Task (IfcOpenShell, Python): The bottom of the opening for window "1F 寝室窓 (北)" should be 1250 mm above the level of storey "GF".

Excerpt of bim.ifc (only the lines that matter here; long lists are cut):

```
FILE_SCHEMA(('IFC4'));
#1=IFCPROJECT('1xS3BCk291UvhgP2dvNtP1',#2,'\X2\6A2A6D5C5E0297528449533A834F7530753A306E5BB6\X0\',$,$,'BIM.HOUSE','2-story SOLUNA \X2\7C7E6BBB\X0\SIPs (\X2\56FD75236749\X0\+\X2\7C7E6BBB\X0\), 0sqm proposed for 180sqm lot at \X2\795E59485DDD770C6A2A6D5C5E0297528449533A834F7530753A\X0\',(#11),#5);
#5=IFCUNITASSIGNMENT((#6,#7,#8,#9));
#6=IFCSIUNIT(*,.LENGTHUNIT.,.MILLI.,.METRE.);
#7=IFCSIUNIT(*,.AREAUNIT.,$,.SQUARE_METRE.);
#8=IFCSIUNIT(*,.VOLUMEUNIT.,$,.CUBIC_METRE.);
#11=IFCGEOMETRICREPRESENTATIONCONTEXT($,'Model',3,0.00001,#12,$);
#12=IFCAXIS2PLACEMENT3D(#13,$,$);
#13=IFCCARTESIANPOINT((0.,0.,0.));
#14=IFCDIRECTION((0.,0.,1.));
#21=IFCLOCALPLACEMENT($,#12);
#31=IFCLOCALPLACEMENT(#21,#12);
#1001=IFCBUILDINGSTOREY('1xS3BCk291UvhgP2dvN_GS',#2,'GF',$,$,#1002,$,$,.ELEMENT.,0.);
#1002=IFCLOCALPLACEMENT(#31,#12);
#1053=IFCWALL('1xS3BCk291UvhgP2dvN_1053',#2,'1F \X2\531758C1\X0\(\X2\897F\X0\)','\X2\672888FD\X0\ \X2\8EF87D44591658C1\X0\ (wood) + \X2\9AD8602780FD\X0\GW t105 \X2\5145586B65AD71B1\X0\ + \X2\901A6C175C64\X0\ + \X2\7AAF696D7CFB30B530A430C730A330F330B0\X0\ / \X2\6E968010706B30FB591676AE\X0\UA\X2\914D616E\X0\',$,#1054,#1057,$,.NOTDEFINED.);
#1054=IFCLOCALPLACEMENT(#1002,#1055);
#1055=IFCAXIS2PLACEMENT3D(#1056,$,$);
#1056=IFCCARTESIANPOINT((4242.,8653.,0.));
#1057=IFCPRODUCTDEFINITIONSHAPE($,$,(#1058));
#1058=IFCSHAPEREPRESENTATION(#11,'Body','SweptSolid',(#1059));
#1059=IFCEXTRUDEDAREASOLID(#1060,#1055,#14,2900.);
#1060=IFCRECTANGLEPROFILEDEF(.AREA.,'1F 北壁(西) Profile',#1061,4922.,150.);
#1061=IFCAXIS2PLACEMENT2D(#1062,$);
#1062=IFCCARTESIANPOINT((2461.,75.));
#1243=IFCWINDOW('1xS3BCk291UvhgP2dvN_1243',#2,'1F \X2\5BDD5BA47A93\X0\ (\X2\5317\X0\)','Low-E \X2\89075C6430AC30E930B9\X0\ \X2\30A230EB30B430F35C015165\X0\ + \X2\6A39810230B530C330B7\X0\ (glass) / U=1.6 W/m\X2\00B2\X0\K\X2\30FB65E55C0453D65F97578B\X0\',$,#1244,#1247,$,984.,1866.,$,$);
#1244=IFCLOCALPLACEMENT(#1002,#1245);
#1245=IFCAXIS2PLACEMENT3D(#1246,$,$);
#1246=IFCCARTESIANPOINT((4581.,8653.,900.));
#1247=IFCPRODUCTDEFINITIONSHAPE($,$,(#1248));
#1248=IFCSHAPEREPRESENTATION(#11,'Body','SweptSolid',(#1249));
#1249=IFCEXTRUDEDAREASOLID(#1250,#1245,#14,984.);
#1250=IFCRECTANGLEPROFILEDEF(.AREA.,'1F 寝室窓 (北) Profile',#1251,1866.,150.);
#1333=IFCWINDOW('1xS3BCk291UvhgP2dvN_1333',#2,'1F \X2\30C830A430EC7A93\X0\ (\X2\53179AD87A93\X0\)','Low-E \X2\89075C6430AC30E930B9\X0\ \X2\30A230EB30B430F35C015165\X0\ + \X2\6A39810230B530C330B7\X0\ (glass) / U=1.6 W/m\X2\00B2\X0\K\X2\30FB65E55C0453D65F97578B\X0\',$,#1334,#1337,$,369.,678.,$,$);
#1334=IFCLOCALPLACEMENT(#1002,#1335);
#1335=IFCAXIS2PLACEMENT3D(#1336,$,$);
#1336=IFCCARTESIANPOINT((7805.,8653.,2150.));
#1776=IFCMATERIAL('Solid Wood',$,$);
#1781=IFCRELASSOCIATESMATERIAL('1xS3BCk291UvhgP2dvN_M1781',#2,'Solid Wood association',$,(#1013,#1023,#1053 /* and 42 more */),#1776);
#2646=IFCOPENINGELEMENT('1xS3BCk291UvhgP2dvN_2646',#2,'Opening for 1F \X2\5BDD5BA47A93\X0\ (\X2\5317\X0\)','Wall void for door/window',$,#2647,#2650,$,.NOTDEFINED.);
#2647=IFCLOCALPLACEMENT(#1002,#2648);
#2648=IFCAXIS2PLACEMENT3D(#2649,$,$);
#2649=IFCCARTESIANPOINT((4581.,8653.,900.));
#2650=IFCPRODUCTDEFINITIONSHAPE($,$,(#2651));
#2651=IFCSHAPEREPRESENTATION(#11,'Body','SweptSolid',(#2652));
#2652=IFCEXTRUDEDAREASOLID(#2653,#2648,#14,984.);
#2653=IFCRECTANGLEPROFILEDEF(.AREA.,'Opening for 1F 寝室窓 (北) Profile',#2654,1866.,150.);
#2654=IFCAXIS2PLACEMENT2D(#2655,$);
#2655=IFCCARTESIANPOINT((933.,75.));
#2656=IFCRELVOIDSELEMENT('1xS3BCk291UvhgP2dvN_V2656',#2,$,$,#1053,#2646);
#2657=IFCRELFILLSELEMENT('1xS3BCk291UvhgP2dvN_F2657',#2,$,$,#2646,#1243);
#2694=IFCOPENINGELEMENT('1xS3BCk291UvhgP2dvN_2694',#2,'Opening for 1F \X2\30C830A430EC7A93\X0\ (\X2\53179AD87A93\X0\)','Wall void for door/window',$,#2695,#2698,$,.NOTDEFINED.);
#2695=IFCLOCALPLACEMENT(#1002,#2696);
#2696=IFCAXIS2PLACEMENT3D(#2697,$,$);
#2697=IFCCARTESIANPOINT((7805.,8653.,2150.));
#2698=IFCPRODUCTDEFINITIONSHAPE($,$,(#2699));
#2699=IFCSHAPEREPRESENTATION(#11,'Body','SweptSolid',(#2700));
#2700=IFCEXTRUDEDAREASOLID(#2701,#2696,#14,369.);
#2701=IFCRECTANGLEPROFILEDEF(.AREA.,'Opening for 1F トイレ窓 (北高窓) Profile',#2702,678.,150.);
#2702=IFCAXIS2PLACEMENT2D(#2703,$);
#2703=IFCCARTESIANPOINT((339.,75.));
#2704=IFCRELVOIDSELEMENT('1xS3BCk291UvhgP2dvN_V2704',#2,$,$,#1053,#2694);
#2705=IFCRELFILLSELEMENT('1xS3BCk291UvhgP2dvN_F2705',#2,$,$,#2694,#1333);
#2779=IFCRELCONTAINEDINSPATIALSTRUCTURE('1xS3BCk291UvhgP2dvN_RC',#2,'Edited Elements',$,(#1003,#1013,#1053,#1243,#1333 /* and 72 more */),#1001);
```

```python
import numpy as np
import ifcopenshell
import ifcopenshell.api.geometry
import ifcopenshell.geom
import ifcopenshell.util.element
import ifcopenshell.util.placement
import ifcopenshell.util.shape
import ifcopenshell.util.unit

model = ifcopenshell.open("bim.ifc")
unit_scale = ifcopenshell.util.unit.calculate_unit_scale(model)

window = model.by_guid("1xS3BCk291UvhgP2dvN_1243")
opening = window.FillsVoids[0].RelatingOpeningElement
storey = ifcopenshell.util.element.get_container(window, ifc_class="IfcBuildingStorey")
level = ifcopenshell.util.placement.get_local_placement(storey.ObjectPlacement)[2, 3]

# The opening's origin need not be at the sill, so measure its lowest point.
shape = ifcopenshell.geom.create_shape(ifcopenshell.geom.settings(), opening)
bottom = ifcopenshell.util.shape.get_shape_bottom_elevation(shape, shape.geometry) / unit_scale
dz = level + 1.25 / unit_scale - bottom

shift = np.array([0.0, 0.0, dz])
# The window is not placed relative to its opening, so move both.
for product in (opening, window):
    matrix = ifcopenshell.util.placement.get_local_placement(product.ObjectPlacement)
    matrix[:3, 3] += shift
    ifcopenshell.api.geometry.edit_object_placement(model, product=product, matrix=matrix, is_si=False)

print(f"moved by {dz * unit_scale:+.3f} m")

model.write("bim_edited.ifc")
```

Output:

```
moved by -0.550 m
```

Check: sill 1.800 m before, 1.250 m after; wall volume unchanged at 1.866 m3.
